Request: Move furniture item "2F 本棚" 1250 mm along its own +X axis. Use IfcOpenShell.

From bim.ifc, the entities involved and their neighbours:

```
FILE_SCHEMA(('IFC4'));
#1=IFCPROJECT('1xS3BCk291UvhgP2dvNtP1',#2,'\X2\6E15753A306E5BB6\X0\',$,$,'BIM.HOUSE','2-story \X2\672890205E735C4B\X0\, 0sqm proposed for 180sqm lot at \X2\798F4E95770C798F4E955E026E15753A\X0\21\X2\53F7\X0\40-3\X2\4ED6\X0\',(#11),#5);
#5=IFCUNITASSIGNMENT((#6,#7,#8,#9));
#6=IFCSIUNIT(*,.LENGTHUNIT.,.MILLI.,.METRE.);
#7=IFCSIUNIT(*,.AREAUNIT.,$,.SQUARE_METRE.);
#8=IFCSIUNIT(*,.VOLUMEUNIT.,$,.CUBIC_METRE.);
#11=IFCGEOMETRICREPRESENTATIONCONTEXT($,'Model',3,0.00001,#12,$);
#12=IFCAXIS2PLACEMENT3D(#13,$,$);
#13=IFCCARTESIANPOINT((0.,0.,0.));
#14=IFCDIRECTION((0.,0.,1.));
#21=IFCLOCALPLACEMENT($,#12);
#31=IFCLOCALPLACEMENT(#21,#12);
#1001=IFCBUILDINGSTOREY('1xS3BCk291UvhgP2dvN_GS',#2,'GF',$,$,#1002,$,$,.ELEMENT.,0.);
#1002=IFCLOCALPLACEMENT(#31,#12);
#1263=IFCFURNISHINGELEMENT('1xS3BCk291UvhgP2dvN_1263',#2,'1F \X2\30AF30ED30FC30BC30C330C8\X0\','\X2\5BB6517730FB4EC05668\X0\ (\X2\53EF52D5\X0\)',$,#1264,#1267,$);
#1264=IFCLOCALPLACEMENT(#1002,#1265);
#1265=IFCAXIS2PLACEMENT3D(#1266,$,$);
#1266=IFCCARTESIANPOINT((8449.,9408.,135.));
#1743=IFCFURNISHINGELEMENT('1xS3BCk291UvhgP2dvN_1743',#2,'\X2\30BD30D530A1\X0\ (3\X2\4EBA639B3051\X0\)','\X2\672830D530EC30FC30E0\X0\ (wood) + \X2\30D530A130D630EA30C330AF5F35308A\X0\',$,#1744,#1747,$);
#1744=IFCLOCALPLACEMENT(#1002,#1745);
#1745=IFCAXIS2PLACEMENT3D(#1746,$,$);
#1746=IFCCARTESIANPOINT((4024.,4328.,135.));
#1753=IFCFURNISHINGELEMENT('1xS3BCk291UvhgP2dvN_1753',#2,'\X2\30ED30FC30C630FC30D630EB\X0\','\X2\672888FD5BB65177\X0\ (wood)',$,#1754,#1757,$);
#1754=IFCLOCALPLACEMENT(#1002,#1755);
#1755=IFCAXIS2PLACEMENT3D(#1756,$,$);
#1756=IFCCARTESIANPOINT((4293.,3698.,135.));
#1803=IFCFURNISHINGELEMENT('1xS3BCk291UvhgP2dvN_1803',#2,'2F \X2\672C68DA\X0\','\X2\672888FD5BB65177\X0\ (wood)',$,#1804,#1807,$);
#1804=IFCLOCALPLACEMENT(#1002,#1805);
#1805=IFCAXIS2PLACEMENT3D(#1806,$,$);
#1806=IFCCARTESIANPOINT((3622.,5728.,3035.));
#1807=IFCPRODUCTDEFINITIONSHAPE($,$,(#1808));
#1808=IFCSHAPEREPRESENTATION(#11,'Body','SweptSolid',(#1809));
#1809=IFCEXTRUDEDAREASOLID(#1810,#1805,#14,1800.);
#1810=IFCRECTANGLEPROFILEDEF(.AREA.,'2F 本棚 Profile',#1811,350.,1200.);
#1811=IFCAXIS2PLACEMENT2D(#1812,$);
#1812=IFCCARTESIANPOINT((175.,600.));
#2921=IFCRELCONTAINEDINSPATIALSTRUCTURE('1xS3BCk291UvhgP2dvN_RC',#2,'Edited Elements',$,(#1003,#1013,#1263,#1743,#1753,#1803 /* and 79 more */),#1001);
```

```python
import ifcopenshell
import ifcopenshell.api.geometry
import ifcopenshell.util.placement
import ifcopenshell.util.unit

model = ifcopenshell.open("bim.ifc")
unit_scale = ifcopenshell.util.unit.calculate_unit_scale(model)

item = model.by_guid("1xS3BCk291UvhgP2dvN_1803")
matrix = ifcopenshell.util.placement.get_local_placement(item.ObjectPlacement)
matrix[:3, 3] += matrix[:3, 0] * 1.25 / unit_scale
ifcopenshell.api.geometry.edit_object_placement(model, product=item, matrix=matrix, is_si=False)

print(ifcopenshell.util.placement.get_local_placement(item.ObjectPlacement).round(3) + 0.0)

model.write("bim_v2.ifc")
```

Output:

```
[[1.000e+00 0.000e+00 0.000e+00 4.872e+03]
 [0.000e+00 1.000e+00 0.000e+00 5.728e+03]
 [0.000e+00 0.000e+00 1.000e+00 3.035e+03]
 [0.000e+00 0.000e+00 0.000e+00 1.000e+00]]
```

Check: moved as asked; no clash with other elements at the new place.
